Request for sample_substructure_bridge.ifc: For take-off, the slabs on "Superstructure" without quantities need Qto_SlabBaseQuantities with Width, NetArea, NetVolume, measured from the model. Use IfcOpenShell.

First a look at what the model holds.

```python
import ifcopenshell
import ifcopenshell.util.element
import ifcopenshell.util.unit

model = ifcopenshell.open("sample_substructure_bridge.ifc")
print(model.schema)
for unit_type in ("LENGTHUNIT", "AREAUNIT", "VOLUMEUNIT"):
    print(unit_type, ifcopenshell.util.unit.calculate_unit_scale(model, unit_type))
storey = next(s for s in model.by_type("IfcBuildingStorey") if s.Name == "Superstructure")
slabs = [e for e in ifcopenshell.util.element.get_decomposition(storey) if e.is_a("IfcSlab")]
for e in sorted(slabs, key=lambda e: e.id()):
    print(e.id(), e.is_a(), e.Name, list(ifcopenshell.util.element.get_psets(e, qtos_only=True)), sep=" | ")
```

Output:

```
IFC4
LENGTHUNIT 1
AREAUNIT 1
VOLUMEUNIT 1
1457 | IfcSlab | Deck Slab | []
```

```python
import ifcopenshell
import ifcopenshell.api.pset
import ifcopenshell.geom
import ifcopenshell.util.element
import ifcopenshell.util.shape
import ifcopenshell.util.unit

model = ifcopenshell.open("sample_substructure_bridge.ifc")
unit_scale = ifcopenshell.util.unit.calculate_unit_scale(model)
area_scale = ifcopenshell.util.unit.calculate_unit_scale(model, "AREAUNIT")
volume_scale = ifcopenshell.util.unit.calculate_unit_scale(model, "VOLUMEUNIT")
settings = ifcopenshell.geom.settings()

storey = next(s for s in model.by_type("IfcBuildingStorey") if s.Name == "Superstructure")
slabs = [e for e in ifcopenshell.util.element.get_decomposition(storey) if e.is_a("IfcSlab")]

for e in sorted(slabs, key=lambda e: e.id()):
    if ifcopenshell.util.element.get_psets(e, qtos_only=True, should_inherit=False):
        continue
    # Geometry comes back in metres, in the element's own axes.
    shape = ifcopenshell.geom.create_shape(settings, e)
    values = {
        "Width": ifcopenshell.util.shape.get_z(shape.geometry) / unit_scale,
        "NetArea": ifcopenshell.util.shape.get_footprint_area(shape.geometry) / area_scale,
        "NetVolume": ifcopenshell.util.shape.get_volume(shape.geometry) / volume_scale,
    }
    qto = ifcopenshell.api.pset.add_qto(model, product=e, name="Qto_SlabBaseQuantities")
    ifcopenshell.api.pset.edit_qto(model, qto=qto, properties=values)
    print(e.id(), {k: round(v, 3) for k, v in values.items()})

model.write("sample_substructure_bridge-out.ifc")
```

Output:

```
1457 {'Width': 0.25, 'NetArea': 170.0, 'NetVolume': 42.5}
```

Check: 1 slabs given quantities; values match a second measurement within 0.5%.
